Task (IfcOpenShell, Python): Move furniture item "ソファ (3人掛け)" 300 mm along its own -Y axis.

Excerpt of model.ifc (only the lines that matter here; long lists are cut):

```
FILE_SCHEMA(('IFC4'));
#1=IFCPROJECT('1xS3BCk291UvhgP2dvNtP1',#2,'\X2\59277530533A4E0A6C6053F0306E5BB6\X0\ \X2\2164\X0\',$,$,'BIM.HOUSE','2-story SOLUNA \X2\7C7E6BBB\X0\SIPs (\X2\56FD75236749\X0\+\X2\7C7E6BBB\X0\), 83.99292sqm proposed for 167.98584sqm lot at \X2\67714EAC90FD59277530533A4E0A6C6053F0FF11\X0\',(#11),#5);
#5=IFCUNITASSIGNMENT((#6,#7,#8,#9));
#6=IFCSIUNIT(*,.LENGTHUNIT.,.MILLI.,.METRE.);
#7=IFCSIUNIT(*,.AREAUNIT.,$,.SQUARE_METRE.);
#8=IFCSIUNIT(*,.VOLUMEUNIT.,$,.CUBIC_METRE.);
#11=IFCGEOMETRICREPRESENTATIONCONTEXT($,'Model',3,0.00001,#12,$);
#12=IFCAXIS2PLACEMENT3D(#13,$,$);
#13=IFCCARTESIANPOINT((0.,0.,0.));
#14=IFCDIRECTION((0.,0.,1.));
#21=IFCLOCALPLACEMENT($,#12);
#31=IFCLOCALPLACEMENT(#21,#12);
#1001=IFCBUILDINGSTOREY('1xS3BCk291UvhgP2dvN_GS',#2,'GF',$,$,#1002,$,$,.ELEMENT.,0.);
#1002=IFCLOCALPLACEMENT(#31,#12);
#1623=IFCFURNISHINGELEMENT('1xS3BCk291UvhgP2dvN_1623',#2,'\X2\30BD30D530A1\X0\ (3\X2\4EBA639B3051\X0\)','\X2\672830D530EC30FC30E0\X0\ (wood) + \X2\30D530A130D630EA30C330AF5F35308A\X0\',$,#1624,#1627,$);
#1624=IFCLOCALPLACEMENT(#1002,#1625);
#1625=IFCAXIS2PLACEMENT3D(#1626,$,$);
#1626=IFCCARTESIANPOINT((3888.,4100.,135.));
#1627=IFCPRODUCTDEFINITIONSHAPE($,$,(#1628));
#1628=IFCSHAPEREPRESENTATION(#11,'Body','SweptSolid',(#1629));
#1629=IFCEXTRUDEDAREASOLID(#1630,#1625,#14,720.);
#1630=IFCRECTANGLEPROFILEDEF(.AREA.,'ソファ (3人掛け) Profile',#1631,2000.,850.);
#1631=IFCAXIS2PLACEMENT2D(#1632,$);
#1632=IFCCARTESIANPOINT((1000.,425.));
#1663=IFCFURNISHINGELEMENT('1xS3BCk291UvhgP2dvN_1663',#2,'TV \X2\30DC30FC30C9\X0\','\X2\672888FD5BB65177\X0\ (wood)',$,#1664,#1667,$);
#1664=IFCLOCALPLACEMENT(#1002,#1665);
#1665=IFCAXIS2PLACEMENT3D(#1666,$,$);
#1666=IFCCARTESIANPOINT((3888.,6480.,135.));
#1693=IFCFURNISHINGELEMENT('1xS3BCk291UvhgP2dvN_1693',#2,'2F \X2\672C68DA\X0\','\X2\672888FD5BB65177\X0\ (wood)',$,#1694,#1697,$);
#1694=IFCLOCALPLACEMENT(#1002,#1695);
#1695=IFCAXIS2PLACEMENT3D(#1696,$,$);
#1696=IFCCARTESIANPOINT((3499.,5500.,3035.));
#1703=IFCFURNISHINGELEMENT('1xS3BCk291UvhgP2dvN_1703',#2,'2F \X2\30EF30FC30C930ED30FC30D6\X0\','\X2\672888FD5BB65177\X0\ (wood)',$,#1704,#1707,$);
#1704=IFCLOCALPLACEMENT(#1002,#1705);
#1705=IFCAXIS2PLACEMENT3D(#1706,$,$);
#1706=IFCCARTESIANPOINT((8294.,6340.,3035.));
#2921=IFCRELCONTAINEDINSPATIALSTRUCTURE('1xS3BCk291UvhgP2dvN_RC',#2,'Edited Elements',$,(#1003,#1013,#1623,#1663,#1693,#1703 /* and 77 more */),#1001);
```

```python
import ifcopenshell
import ifcopenshell.api.geometry
import ifcopenshell.util.placement
import ifcopenshell.util.unit

model = ifcopenshell.open("model.ifc")
unit_scale = ifcopenshell.util.unit.calculate_unit_scale(model)

item = model.by_guid("1xS3BCk291UvhgP2dvN_1623")
matrix = ifcopenshell.util.placement.get_local_placement(item.ObjectPlacement)
matrix[:3, 3] -= matrix[:3, 1] * 0.3 / unit_scale
ifcopenshell.api.geometry.edit_object_placement(model, product=item, matrix=matrix, is_si=False)

print(ifcopenshell.util.placement.get_local_placement(item.ObjectPlacement).round(3) + 0.0)

model.write("model_v2.ifc")
```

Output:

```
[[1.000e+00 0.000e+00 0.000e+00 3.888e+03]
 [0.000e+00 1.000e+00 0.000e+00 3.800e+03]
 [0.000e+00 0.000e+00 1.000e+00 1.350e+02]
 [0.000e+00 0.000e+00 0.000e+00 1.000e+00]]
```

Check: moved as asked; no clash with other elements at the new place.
